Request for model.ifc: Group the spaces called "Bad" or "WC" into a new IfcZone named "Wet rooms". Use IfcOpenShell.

First a look at what the model holds.

```python
import ifcopenshell

model = ifcopenshell.open("model.ifc")
print(model.schema)
seen = {}
for space in model.by_type("IfcSpace"):
    seen[space.LongName] = seen.get(space.LongName, 0) + 1
for name, count in sorted(seen.items(), key=str):
    print(count, "x", name)
print("zones:", [z.Name for z in model.by_type("IfcZone")][:20])
```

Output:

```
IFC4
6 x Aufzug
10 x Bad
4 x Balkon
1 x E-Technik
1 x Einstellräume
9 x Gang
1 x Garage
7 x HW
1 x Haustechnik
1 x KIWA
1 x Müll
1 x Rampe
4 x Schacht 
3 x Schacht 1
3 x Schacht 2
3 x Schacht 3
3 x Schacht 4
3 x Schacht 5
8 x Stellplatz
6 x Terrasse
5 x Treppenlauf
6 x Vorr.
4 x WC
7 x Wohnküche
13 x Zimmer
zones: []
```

```python
import ifcopenshell
import ifcopenshell.api.group
import ifcopenshell.api.root

model = ifcopenshell.open("model.ifc")

names = {"Bad", "WC"}
spaces = [s for s in model.by_type("IfcSpace") if s.LongName in names]

zone = ifcopenshell.api.root.create_entity(model, ifc_class="IfcZone", name="Wet rooms")
ifcopenshell.api.group.assign_group(model, products=spaces, group=zone)
print(len(spaces), "spaces in", zone.Name)

model.write("model-out.ifc")
```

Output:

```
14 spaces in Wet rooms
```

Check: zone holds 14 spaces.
